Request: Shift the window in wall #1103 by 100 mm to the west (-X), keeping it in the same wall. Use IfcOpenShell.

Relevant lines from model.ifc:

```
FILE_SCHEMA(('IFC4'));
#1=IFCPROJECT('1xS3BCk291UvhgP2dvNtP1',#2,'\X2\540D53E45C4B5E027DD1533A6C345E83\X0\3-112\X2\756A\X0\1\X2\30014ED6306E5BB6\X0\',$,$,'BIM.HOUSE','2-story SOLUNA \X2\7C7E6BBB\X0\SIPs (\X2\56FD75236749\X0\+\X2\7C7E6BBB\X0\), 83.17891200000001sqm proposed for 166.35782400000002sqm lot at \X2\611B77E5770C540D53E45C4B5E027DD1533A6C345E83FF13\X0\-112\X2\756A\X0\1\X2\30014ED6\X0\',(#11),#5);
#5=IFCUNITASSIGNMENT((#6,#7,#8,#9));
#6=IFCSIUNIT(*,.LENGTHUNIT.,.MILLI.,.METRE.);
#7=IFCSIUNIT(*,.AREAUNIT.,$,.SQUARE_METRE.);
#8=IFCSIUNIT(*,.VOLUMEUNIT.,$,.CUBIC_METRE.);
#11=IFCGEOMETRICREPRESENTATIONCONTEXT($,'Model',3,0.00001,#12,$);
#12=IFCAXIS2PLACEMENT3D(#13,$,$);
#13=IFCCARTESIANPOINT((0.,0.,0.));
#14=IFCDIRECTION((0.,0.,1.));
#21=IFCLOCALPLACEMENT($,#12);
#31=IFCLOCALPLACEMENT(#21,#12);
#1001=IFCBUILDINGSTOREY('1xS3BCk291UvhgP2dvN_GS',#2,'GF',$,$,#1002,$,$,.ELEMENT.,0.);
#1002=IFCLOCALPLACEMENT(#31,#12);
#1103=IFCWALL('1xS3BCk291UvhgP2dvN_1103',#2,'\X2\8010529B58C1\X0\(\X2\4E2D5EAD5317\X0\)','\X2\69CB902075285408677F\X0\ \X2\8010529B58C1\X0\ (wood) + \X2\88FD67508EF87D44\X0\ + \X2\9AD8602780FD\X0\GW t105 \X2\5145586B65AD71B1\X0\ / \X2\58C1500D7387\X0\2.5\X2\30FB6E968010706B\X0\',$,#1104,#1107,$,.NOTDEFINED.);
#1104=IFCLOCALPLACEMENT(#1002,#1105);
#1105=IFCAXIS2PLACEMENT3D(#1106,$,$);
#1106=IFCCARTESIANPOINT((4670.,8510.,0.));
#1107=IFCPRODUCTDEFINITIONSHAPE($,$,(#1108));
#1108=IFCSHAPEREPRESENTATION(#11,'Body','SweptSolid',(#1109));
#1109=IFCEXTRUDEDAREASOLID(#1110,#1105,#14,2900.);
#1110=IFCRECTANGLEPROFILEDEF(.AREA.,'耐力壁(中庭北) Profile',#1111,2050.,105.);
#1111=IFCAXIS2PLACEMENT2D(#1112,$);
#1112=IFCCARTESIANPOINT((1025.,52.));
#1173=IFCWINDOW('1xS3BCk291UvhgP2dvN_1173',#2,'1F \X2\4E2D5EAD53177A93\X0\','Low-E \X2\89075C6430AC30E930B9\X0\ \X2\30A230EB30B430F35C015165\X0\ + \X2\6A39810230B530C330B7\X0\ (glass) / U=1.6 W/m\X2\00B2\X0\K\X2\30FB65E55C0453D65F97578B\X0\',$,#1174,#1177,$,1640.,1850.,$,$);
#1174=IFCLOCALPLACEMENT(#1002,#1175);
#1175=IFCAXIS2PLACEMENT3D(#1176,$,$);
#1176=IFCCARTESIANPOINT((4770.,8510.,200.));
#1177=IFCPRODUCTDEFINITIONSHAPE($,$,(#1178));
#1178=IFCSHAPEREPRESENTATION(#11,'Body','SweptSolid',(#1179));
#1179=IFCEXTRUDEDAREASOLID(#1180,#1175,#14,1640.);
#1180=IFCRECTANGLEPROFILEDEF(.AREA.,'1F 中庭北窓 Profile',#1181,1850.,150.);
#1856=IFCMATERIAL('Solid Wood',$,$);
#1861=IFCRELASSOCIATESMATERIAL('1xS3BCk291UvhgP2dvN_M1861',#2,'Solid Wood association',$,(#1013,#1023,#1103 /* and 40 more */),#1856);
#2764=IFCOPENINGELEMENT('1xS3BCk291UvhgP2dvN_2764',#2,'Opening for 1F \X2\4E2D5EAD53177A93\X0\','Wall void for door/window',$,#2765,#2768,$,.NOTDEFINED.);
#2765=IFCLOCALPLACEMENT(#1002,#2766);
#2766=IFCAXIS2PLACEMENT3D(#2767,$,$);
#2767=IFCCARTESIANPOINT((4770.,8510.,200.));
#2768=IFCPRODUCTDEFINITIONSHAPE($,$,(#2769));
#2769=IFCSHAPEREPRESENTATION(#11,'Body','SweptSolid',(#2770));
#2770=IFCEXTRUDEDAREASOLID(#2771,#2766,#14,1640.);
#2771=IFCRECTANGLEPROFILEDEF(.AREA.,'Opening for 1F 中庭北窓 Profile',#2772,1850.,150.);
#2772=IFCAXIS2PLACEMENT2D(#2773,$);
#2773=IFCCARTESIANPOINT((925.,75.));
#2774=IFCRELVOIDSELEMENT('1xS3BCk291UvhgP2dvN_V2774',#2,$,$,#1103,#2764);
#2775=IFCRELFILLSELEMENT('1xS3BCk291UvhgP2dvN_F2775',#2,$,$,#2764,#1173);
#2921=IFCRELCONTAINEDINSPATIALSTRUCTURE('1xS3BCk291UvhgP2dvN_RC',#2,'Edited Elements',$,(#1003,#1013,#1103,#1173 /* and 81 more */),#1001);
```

```python
import ifcopenshell
import ifcopenshell.api.geometry
import ifcopenshell.util.placement
import ifcopenshell.util.unit

model = ifcopenshell.open("model.ifc")
unit_scale = ifcopenshell.util.unit.calculate_unit_scale(model)

window = model.by_guid("1xS3BCk291UvhgP2dvN_1173")
opening = window.FillsVoids[0].RelatingOpeningElement
wall = opening.VoidsElements[0].RelatingBuildingElement

wall_matrix = ifcopenshell.util.placement.get_local_placement(wall.ObjectPlacement)
shift = wall_matrix[:3, 0] * -0.1 / unit_scale
before = ifcopenshell.util.placement.get_local_placement(window.ObjectPlacement)[:3, 3].copy()

# The window is not placed relative to its opening, so move both.
for product in (opening, window):
    matrix = ifcopenshell.util.placement.get_local_placement(product.ObjectPlacement)
    matrix[:3, 3] += shift
    ifcopenshell.api.geometry.edit_object_placement(model, product=product, matrix=matrix, is_si=False)

after = ifcopenshell.util.placement.get_local_placement(window.ObjectPlacement)[:3, 3]
print("window moved by", (after - before).round(3) + 0.0)

model.write("model_updated.ifc")
```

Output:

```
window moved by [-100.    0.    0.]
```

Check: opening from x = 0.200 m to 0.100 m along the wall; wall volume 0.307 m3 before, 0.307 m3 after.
